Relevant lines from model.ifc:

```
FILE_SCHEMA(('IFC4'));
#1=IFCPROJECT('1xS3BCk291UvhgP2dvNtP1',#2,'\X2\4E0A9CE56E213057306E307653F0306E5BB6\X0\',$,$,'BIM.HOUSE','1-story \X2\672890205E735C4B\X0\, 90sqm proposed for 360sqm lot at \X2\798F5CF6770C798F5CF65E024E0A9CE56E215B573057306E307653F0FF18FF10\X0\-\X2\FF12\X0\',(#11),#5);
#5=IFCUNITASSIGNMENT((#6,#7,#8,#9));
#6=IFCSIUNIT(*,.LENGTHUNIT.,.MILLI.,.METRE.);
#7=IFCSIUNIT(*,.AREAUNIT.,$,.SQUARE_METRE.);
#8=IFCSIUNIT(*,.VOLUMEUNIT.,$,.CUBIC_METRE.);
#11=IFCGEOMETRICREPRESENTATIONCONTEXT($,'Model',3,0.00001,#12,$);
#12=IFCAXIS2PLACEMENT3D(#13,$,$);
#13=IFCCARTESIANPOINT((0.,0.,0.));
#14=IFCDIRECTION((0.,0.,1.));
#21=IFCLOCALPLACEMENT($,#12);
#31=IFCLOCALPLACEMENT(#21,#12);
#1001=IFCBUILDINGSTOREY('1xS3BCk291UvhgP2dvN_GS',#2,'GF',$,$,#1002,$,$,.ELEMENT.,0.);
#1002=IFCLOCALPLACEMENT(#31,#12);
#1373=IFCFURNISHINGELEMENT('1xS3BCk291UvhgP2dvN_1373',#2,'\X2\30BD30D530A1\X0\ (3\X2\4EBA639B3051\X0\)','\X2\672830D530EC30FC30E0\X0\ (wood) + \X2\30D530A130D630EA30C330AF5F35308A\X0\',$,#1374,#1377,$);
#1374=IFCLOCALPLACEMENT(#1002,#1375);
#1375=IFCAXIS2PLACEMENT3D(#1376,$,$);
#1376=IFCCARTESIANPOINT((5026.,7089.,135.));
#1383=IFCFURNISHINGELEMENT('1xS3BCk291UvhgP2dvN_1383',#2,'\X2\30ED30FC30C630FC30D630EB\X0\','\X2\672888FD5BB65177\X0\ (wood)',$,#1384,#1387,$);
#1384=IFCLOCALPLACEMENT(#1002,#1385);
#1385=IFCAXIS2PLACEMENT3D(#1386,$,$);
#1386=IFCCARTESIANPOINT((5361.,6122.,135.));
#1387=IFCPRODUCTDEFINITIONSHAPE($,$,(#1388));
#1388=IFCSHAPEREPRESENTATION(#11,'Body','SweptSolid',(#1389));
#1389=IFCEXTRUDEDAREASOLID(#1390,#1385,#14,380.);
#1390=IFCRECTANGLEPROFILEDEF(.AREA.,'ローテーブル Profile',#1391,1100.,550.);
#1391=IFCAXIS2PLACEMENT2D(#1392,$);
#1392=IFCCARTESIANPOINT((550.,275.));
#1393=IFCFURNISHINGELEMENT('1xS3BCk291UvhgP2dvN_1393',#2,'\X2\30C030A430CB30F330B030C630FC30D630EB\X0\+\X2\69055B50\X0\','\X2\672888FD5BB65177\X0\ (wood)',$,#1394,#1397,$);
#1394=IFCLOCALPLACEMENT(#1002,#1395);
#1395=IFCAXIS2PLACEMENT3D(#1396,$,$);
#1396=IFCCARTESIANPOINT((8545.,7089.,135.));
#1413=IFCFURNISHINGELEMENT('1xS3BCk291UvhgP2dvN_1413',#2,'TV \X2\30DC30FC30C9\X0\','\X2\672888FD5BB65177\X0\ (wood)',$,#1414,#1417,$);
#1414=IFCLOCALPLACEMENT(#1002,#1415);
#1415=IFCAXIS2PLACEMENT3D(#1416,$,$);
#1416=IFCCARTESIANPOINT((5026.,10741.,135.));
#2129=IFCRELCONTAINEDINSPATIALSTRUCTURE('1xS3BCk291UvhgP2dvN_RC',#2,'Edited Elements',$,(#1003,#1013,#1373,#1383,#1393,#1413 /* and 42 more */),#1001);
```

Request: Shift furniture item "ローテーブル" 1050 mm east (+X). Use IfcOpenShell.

```python
import ifcopenshell
import ifcopenshell.api.geometry
import ifcopenshell.util.placement
import ifcopenshell.util.unit

model = ifcopenshell.open("model.ifc")
unit_scale = ifcopenshell.util.unit.calculate_unit_scale(model)

item = model.by_guid("1xS3BCk291UvhgP2dvN_1383")
matrix = ifcopenshell.util.placement.get_local_placement(item.ObjectPlacement)
matrix[0, 3] += 1.05 / unit_scale
ifcopenshell.api.geometry.edit_object_placement(model, product=item, matrix=matrix, is_si=False)

print(ifcopenshell.util.placement.get_local_placement(item.ObjectPlacement).round(3) + 0.0)

model.write("model_v2.ifc")
```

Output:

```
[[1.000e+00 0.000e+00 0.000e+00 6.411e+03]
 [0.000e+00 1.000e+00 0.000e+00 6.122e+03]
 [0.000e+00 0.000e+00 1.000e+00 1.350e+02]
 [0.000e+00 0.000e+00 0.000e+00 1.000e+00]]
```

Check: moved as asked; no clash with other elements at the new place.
